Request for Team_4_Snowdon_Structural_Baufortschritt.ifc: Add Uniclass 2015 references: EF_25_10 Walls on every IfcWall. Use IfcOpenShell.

First a look at what the model holds.

```python
import ifcopenshell

model = ifcopenshell.open("Team_4_Snowdon_Structural_Baufortschritt.ifc")
print(model.schema)
print("classifications:", [c.Name for c in model.by_type("IfcClassification")])
for ifc_class in ("IfcDoor", "IfcRoof", "IfcStair", "IfcWall", "IfcWindow"):
    print(ifc_class, len(model.by_type(ifc_class)))
```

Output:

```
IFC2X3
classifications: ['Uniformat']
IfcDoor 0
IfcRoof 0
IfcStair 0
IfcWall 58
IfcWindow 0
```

```python
import ifcopenshell
import ifcopenshell.api.classification

model = ifcopenshell.open("Team_4_Snowdon_Structural_Baufortschritt.ifc")

# IFC2X3 requires Source and Edition and has no link from the project to the system.
system = model.create_entity("IfcClassification", Source="NBS", Edition="2015", Name="Uniclass 2015")

codes = {
    "IfcWall": ("EF_25_10", "Walls"),
}
for ifc_class, (code, name) in codes.items():
    products = model.by_type(ifc_class)
    ifcopenshell.api.classification.add_reference(
        model, products=products, classification=system, identification=code, name=name
    )
    print(code, len(products))

model.write("Team_4_Snowdon_Structural_Baufortschritt_edited.ifc")
```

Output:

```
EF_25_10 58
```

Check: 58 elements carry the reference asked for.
